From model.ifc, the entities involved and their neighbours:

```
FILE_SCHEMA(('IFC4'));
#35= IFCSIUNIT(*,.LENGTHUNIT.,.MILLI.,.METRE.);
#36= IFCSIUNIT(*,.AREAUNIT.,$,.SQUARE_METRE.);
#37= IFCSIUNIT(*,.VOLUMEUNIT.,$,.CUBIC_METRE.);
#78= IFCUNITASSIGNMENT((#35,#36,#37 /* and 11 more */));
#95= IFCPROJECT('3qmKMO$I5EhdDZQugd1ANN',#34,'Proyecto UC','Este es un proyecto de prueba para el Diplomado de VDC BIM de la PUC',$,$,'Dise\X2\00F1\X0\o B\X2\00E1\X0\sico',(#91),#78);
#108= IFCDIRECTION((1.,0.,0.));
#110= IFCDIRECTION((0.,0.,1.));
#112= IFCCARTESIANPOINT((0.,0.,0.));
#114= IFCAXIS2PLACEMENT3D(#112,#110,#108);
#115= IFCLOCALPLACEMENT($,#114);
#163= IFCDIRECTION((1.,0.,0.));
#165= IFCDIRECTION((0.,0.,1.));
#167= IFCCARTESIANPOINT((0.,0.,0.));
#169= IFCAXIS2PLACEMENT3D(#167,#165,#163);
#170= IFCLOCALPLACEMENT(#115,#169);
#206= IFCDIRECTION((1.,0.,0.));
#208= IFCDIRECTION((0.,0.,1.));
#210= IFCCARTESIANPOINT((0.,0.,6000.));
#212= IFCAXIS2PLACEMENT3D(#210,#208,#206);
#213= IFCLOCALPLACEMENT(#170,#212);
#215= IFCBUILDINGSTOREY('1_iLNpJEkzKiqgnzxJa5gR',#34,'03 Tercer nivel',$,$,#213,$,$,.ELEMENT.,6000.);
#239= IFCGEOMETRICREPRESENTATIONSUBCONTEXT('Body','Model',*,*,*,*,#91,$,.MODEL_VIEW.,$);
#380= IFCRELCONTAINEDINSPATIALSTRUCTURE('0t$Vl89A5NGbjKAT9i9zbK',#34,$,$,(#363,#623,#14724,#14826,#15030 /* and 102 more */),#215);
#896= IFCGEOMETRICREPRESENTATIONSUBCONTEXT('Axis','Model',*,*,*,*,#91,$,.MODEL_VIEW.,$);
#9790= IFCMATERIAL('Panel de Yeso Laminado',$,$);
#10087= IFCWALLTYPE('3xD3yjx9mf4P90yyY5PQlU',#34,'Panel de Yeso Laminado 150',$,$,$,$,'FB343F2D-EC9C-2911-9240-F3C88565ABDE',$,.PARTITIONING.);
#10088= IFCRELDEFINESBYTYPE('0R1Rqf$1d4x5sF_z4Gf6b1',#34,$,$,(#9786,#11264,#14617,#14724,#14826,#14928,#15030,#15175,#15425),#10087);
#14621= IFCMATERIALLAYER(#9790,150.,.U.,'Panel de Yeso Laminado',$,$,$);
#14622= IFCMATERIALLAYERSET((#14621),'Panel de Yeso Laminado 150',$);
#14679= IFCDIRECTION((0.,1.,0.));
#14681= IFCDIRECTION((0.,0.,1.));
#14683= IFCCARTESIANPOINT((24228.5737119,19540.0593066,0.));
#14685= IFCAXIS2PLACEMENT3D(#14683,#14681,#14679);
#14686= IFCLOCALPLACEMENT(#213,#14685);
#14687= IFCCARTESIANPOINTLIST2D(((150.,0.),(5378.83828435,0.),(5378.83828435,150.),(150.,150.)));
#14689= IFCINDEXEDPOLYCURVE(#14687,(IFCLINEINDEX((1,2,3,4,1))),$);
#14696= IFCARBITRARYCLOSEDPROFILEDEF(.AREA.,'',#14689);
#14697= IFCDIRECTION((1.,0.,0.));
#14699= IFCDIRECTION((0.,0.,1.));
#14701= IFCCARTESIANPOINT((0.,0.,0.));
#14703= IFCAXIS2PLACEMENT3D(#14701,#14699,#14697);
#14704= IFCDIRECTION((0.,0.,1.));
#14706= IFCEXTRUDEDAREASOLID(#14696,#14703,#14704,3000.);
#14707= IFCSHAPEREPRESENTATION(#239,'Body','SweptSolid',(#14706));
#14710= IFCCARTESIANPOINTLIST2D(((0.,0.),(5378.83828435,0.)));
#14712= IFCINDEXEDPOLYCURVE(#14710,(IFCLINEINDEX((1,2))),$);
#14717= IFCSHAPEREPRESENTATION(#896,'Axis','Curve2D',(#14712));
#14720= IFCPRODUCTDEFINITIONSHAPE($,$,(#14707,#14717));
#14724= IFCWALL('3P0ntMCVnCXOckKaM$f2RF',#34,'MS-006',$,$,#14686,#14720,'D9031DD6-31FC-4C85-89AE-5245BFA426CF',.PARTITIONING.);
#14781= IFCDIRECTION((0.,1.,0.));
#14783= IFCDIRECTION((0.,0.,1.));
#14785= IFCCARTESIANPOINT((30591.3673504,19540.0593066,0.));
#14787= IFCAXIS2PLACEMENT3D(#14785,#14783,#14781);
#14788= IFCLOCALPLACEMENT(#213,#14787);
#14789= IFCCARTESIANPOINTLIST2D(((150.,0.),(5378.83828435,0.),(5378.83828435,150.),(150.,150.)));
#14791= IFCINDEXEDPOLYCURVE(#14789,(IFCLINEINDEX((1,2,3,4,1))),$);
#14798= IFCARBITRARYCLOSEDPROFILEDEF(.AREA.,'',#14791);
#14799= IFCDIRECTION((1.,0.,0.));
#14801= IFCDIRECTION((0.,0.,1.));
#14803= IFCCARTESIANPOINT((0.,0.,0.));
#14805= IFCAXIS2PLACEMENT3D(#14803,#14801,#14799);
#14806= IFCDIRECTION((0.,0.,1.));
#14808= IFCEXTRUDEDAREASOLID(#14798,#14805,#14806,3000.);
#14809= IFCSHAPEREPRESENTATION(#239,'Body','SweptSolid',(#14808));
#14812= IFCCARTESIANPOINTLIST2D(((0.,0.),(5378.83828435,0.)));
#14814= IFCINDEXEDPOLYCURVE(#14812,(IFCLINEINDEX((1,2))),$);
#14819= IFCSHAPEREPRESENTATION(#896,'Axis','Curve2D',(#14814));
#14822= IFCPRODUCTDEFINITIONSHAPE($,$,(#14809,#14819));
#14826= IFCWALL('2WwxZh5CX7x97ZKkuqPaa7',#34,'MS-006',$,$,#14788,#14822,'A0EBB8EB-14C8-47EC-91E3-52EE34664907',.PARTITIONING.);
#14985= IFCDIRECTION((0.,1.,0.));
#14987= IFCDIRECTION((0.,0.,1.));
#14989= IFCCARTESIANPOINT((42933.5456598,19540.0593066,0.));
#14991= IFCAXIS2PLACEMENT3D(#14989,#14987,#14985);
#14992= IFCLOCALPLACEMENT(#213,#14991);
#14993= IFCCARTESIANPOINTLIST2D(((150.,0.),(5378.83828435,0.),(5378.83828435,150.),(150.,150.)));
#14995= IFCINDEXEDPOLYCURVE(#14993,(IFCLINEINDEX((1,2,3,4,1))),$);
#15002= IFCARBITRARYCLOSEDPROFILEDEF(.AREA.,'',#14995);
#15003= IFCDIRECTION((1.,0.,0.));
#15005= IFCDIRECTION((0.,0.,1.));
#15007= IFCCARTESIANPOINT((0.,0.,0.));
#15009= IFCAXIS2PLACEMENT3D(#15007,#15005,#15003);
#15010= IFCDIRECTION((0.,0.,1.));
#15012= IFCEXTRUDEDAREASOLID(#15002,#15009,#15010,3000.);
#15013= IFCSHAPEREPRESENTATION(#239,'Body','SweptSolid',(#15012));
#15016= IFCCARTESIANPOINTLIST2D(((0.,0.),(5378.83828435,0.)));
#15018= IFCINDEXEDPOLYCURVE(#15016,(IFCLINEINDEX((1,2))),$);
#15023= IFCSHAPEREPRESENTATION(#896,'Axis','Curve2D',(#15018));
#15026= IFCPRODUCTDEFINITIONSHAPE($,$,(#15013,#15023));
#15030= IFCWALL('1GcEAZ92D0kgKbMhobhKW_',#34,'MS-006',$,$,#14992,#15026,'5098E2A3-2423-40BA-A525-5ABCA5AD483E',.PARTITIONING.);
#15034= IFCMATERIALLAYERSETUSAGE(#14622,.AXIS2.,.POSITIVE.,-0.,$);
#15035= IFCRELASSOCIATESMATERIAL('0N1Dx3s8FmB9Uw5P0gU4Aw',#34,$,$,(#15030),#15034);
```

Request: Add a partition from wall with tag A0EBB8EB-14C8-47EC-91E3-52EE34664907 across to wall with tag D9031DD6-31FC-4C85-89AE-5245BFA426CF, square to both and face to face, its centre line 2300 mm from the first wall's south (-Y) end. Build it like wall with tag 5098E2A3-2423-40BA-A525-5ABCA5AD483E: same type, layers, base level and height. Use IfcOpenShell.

```python
import numpy as np
import ifcopenshell
import ifcopenshell.api.geometry
import ifcopenshell.api.material
import ifcopenshell.api.pset
import ifcopenshell.api.root
import ifcopenshell.api.spatial
import ifcopenshell.api.type
import ifcopenshell.geom
import ifcopenshell.util.element
import ifcopenshell.util.placement
import ifcopenshell.util.representation
import ifcopenshell.util.shape
import ifcopenshell.util.unit

model = ifcopenshell.open("model.ifc")
unit_scale = ifcopenshell.util.unit.calculate_unit_scale(model)
settings = ifcopenshell.geom.settings()
settings.set("use-world-coords", True)

start_wall = model.by_guid("2WwxZh5CX7x97ZKkuqPaa7")
end_wall = model.by_guid("3P0ntMCVnCXOckKaM$f2RF")
like = model.by_id(15030)
matrix = ifcopenshell.util.placement.get_local_placement(start_wall.ObjectPlacement)
matrix[:3, 3] *= unit_scale


def extent(element):
    """Bounding box in the first wall's axes, in metres."""
    shape = ifcopenshell.geom.create_shape(settings, element)
    points = (ifcopenshell.util.shape.get_vertices(shape.geometry) - matrix[:3, 3]) @ matrix[:3, :3]
    return points.min(axis=0), points.max(axis=0)


y_start = extent(start_wall)[1][1]
y_end = extent(end_wall)[0][1]
like_min, like_max = extent(like)
length, height = float(abs(y_end - y_start)), float(like_max[2] - like_min[2])
layer_set = ifcopenshell.util.element.get_material(like, should_skip_usage=True)
thickness = sum(layer.LayerThickness for layer in layer_set.MaterialLayers) * unit_scale

wall = ifcopenshell.api.root.create_entity(model, ifc_class="IfcWall", name="New partition")
storey = ifcopenshell.util.element.get_container(like)
ifcopenshell.api.spatial.assign_container(model, products=[wall], relating_structure=storey)
ifcopenshell.api.type.assign_type(
    model, related_objects=[wall], relating_type=ifcopenshell.util.element.get_type(like), should_map_representations=False
)
rel = ifcopenshell.api.material.assign_material(
    model, products=[wall], type="IfcMaterialLayerSetUsage", material=layer_set
)
rel.RelatingMaterial.OffsetFromReferenceLine = -thickness / 2 / unit_scale
pset = ifcopenshell.api.pset.add_pset(model, product=wall, name="Pset_WallCommon")
ifcopenshell.api.pset.edit_pset(model, pset=pset, properties={"IsExternal": False, "LoadBearing": False})

# The axis runs down the middle of the wall.
axis = ifcopenshell.api.geometry.add_axis_representation(
    model, context=ifcopenshell.util.representation.get_context(model, "Model", "Axis"), axis=[(0.0, 0.0), (length, 0.0)]
)
body = ifcopenshell.api.geometry.add_wall_representation(
    model,
    context=ifcopenshell.util.representation.get_context(model, "Model", "Body", "MODEL_VIEW"),
    length=length,
    height=height,
    thickness=thickness,
    offset=-thickness / 2,
)
for representation in (axis, body):
    ifcopenshell.api.geometry.assign_representation(model, product=wall, representation=representation)

placement = matrix @ ifcopenshell.util.placement.rotation(90, "Z")
placement[:, 3] = matrix @ np.array([extent(start_wall)[0][0] + 2.3, y_start, like_min[2], 1.0])
ifcopenshell.api.geometry.edit_object_placement(model, product=wall, matrix=placement)

print(f"partition {length:.3f} m long, {height:.3f} m high, {thickness:.3f} m thick")

model.write("model-out.ifc")
```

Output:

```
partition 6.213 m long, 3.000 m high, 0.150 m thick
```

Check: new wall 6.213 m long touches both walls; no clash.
